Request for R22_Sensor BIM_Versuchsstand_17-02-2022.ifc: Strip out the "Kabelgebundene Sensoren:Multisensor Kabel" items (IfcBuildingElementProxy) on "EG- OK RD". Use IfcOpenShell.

First a look at what the model holds.

```python
import ifcopenshell
import ifcopenshell.util.element

model = ifcopenshell.open("R22_Sensor BIM_Versuchsstand_17-02-2022.ifc")
print(model.schema)
storey = next(s for s in model.by_type("IfcBuildingStorey") if s.Name == "EG- OK RD")
proxies = [e for e in ifcopenshell.util.element.get_decomposition(storey) if e.is_a("IfcBuildingElementProxy")]
seen = {}
for e in proxies:
    element_type = ifcopenshell.util.element.get_type(e)
    name = element_type.Name if element_type not in (None, e) else None
    seen[name] = seen.get(name, 0) + 1
for name, count in sorted(seen.items(), key=str):
    print(count, "x", name)
```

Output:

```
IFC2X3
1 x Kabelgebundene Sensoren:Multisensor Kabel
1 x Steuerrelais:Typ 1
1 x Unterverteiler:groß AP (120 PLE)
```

```python
import ifcopenshell
import ifcopenshell.api.root
import ifcopenshell.util.element

model = ifcopenshell.open("R22_Sensor BIM_Versuchsstand_17-02-2022.ifc")

storey = next(s for s in model.by_type("IfcBuildingStorey") if s.Name == "EG- OK RD")
proxies = [e for e in ifcopenshell.util.element.get_decomposition(storey) if e.is_a("IfcBuildingElementProxy")]
targets = [e for e in proxies if (t := ifcopenshell.util.element.get_type(e)) not in (None, e) and t.Name == "Kabelgebundene Sensoren:Multisensor Kabel"]

for e in targets:
    ifcopenshell.api.root.remove_product(model, product=e)
print(len(targets), "removed")

model.write("R22_Sensor BIM_Versuchsstand_17-02-2022_edited.ifc")
```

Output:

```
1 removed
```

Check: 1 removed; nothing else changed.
